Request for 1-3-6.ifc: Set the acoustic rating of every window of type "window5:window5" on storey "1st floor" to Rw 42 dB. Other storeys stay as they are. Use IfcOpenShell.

First a look at what the model holds.

```python
import ifcopenshell
import ifcopenshell.util.element

model = ifcopenshell.open("1-3-6.ifc")
print(model.schema)
storey = next(s for s in model.by_type("IfcBuildingStorey") if s.Name == "1st floor")
windows = [e for e in ifcopenshell.util.element.get_decomposition(storey) if e.is_a("IfcWindow")]
seen = {}
for e in windows:
    element_type = ifcopenshell.util.element.get_type(e)
    key = (element_type.Name if element_type != e and element_type else None, ifcopenshell.util.element.get_pset(e, "Pset_WindowCommon", "AcousticRating"))
    seen[key] = seen.get(key, 0) + 1
for (name, value), count in sorted(seen.items(), key=str):
    print(count, "x", name, "|", value)
```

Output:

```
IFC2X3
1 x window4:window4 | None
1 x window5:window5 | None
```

```python
import ifcopenshell
import ifcopenshell.api.pset
import ifcopenshell.util.element

model = ifcopenshell.open("1-3-6.ifc")

storey = next(s for s in model.by_type("IfcBuildingStorey") if s.Name == "1st floor")
windows = [e for e in ifcopenshell.util.element.get_decomposition(storey) if e.is_a("IfcWindow")]

count = 0
for e in windows:
    element_type = ifcopenshell.util.element.get_type(e)
    if element_type in (None, e) or element_type.Name != "window5:window5":
        continue
    # add_pset returns the element's existing set when there is one.
    pset = ifcopenshell.api.pset.add_pset(model, product=e, name="Pset_WindowCommon")
    ifcopenshell.api.pset.edit_pset(model, pset=pset, properties={"AcousticRating": "Rw 42 dB"})
    count += 1

print(count, "windows updated")

model.write("1-3-6_v2.ifc")
```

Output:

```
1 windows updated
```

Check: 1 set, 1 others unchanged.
